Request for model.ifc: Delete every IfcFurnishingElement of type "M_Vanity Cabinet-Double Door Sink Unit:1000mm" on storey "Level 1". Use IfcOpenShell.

First a look at what the model holds.

```python
import ifcopenshell
import ifcopenshell.util.element

model = ifcopenshell.open("model.ifc")
print(model.schema)
storey = next(s for s in model.by_type("IfcBuildingStorey") if s.Name == "Level 1")
furniture = [e for e in ifcopenshell.util.element.get_decomposition(storey) if e.is_a("IfcFurnishingElement")]
seen = {}
for e in furniture:
    element_type = ifcopenshell.util.element.get_type(e)
    name = element_type.Name if element_type not in (None, e) else None
    seen[name] = seen.get(name, 0) + 1
for name, count in sorted(seen.items(), key=str):
    print(count, "x", name)
```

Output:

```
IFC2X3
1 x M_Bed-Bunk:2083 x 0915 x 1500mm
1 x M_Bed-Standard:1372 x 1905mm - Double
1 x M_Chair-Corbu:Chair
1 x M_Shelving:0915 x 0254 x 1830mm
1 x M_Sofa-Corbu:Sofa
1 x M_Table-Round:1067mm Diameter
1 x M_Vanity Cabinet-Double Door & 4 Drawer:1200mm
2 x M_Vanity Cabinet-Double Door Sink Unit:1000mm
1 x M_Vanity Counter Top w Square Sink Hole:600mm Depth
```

```python
import ifcopenshell
import ifcopenshell.api.root
import ifcopenshell.util.element

model = ifcopenshell.open("model.ifc")

storey = next(s for s in model.by_type("IfcBuildingStorey") if s.Name == "Level 1")
furniture = [e for e in ifcopenshell.util.element.get_decomposition(storey) if e.is_a("IfcFurnishingElement")]
targets = [e for e in furniture if (t := ifcopenshell.util.element.get_type(e)) not in (None, e) and t.Name == "M_Vanity Cabinet-Double Door Sink Unit:1000mm"]

for e in targets:
    ifcopenshell.api.root.remove_product(model, product=e)
print(len(targets), "removed")

model.write("model-out.ifc")
```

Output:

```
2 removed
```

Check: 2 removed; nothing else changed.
